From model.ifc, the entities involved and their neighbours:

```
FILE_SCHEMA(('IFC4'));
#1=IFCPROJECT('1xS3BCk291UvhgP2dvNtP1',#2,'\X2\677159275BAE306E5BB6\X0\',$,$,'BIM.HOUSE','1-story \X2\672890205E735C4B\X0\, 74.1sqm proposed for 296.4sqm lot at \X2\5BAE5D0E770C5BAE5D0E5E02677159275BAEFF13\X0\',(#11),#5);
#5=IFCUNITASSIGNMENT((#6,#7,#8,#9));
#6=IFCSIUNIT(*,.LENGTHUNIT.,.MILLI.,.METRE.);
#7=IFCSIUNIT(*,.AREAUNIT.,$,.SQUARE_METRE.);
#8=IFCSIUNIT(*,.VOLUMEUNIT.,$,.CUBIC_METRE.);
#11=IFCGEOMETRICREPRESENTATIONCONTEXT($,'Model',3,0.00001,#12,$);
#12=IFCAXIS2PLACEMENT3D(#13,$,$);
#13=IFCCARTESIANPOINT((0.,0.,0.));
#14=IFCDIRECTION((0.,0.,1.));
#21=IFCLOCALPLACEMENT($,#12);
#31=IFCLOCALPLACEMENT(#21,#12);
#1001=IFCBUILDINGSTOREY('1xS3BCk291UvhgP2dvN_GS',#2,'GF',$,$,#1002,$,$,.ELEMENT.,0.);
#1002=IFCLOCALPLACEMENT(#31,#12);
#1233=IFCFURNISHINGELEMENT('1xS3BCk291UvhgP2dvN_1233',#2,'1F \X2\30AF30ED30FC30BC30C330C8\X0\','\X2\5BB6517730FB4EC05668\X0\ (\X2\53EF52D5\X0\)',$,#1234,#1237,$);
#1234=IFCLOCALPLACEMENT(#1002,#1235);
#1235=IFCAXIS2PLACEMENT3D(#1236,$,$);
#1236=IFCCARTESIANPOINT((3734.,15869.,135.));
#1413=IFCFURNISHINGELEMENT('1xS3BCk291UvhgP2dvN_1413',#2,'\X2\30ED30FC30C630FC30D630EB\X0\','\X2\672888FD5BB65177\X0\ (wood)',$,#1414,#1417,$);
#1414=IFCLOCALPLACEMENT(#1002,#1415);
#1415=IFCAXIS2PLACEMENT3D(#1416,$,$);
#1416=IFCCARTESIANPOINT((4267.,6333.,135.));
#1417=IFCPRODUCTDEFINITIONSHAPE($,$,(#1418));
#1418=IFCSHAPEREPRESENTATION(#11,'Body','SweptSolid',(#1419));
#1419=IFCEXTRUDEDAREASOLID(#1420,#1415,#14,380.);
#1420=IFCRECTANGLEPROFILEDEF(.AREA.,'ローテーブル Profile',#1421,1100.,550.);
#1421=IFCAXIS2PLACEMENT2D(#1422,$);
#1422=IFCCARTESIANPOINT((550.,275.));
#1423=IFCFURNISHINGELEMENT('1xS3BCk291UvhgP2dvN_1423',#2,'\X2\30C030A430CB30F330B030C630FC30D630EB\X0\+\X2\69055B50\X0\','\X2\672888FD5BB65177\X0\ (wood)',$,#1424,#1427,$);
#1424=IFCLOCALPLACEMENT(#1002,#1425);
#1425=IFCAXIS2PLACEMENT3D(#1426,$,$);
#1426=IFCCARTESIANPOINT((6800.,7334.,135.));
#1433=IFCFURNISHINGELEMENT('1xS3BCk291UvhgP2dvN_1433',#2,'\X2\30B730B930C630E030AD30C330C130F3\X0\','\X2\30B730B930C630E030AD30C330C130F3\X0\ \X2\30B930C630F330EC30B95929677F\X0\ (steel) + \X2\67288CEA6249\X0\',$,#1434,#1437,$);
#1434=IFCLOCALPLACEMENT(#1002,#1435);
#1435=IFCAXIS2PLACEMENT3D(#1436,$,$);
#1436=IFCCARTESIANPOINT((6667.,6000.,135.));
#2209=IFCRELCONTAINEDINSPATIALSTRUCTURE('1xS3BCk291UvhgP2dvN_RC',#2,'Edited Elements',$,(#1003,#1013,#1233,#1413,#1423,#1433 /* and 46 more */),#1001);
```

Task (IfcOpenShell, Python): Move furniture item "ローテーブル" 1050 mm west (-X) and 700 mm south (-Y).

```python
import ifcopenshell
import ifcopenshell.api.geometry
import ifcopenshell.util.placement

model = ifcopenshell.open("model.ifc")

item = model.by_id(1413)
matrix = ifcopenshell.util.placement.get_local_placement(item.ObjectPlacement)
matrix[0, 3] -= 1050.0
matrix[1, 3] -= 700.0
ifcopenshell.api.geometry.edit_object_placement(model, product=item, matrix=matrix, is_si=False)

print(ifcopenshell.util.placement.get_local_placement(item.ObjectPlacement).round(3) + 0.0)

model.write("model_edited.ifc")
```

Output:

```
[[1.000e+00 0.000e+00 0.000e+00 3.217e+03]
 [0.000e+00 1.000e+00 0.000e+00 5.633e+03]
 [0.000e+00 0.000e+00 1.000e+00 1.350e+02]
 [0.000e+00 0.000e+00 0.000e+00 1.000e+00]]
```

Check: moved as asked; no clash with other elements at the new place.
